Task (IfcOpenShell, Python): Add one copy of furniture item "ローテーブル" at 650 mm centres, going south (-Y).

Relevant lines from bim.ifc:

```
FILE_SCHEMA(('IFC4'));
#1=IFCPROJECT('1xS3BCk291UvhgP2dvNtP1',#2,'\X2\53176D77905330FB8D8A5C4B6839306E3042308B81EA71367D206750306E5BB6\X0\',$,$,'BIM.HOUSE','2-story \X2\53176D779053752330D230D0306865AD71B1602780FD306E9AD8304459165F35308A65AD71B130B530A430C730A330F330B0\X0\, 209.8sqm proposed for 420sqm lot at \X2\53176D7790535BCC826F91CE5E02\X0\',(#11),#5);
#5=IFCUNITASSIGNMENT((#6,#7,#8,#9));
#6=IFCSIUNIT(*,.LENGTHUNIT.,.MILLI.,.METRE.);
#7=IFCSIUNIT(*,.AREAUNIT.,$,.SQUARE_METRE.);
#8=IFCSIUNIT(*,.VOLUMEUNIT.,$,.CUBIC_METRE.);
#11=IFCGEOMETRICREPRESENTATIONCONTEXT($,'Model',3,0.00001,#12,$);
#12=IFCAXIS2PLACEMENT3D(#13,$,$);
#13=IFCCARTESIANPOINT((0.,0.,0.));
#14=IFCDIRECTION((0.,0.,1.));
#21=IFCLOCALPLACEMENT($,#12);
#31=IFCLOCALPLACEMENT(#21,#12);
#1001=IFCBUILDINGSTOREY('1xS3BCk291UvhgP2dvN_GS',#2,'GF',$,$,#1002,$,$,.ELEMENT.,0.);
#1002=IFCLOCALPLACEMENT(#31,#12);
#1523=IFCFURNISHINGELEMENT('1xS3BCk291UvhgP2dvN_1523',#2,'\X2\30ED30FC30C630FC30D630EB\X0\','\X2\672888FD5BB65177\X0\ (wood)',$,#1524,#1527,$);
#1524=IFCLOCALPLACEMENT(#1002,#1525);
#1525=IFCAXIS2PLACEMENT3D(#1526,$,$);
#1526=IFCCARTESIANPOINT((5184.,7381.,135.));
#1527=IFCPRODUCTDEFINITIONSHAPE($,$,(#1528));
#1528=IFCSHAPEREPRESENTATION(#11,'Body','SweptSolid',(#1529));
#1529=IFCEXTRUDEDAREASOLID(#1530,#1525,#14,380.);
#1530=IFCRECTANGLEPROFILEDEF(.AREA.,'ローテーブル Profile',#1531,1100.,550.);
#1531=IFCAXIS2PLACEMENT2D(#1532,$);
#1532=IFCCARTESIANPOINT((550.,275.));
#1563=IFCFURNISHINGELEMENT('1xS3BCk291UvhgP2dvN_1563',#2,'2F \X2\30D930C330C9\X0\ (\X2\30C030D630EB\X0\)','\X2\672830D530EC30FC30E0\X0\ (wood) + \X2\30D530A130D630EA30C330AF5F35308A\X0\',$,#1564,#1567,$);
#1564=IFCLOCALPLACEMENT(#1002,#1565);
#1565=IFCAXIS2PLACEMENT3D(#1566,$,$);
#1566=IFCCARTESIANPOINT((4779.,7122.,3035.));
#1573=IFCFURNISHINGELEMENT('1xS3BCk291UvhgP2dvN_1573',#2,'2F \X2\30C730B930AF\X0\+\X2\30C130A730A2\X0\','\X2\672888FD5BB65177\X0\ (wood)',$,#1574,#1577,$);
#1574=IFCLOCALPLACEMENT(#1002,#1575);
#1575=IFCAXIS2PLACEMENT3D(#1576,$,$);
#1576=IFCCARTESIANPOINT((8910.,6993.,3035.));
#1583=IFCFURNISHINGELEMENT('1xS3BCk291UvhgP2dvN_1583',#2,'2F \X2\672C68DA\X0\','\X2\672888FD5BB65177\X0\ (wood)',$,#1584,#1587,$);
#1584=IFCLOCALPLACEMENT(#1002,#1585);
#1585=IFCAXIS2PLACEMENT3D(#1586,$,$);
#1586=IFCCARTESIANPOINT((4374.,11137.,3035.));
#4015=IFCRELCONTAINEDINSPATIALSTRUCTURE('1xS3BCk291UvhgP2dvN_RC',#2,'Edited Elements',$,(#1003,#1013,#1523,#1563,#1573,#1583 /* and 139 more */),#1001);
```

```python
import numpy as np
import ifcopenshell
import ifcopenshell.api.geometry
import ifcopenshell.api.root
import ifcopenshell.util.element
import ifcopenshell.util.placement

model = ifcopenshell.open("bim.ifc")


def reuse_history(source, copy):
    """copy_class also copies each property set's owner history, people and application; keep the originals."""
    for rel in copy.IsDefinedBy:
        if rel.is_a("IfcRelDefinesByProperties") and (history := rel.RelatingPropertyDefinition.OwnerHistory):
            rel.RelatingPropertyDefinition.OwnerHistory = source.OwnerHistory
            ifcopenshell.util.element.remove_deep2(model, history)


source = model.by_id(1523)
base = ifcopenshell.util.placement.get_local_placement(source.ObjectPlacement)
step = np.array([0.0, -1.0, 0.0]) * 650.0

for i in range(1, 2):
    copy = ifcopenshell.api.root.copy_class(model, product=source)
    copy.Representation = ifcopenshell.util.element.copy_deep(
        model, source.Representation, exclude=["IfcGeometricRepresentationContext", "IfcRepresentationMap"]
    )
    reuse_history(source, copy)
    matrix = base.copy()
    matrix[:3, 3] += i * step
    print("added at", matrix[:3, 3].round(3) + 0.0)
    ifcopenshell.api.geometry.edit_object_placement(model, product=copy, matrix=matrix, is_si=False)

model.write("bim_edited.ifc")
```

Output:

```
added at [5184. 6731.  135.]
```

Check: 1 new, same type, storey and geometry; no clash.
